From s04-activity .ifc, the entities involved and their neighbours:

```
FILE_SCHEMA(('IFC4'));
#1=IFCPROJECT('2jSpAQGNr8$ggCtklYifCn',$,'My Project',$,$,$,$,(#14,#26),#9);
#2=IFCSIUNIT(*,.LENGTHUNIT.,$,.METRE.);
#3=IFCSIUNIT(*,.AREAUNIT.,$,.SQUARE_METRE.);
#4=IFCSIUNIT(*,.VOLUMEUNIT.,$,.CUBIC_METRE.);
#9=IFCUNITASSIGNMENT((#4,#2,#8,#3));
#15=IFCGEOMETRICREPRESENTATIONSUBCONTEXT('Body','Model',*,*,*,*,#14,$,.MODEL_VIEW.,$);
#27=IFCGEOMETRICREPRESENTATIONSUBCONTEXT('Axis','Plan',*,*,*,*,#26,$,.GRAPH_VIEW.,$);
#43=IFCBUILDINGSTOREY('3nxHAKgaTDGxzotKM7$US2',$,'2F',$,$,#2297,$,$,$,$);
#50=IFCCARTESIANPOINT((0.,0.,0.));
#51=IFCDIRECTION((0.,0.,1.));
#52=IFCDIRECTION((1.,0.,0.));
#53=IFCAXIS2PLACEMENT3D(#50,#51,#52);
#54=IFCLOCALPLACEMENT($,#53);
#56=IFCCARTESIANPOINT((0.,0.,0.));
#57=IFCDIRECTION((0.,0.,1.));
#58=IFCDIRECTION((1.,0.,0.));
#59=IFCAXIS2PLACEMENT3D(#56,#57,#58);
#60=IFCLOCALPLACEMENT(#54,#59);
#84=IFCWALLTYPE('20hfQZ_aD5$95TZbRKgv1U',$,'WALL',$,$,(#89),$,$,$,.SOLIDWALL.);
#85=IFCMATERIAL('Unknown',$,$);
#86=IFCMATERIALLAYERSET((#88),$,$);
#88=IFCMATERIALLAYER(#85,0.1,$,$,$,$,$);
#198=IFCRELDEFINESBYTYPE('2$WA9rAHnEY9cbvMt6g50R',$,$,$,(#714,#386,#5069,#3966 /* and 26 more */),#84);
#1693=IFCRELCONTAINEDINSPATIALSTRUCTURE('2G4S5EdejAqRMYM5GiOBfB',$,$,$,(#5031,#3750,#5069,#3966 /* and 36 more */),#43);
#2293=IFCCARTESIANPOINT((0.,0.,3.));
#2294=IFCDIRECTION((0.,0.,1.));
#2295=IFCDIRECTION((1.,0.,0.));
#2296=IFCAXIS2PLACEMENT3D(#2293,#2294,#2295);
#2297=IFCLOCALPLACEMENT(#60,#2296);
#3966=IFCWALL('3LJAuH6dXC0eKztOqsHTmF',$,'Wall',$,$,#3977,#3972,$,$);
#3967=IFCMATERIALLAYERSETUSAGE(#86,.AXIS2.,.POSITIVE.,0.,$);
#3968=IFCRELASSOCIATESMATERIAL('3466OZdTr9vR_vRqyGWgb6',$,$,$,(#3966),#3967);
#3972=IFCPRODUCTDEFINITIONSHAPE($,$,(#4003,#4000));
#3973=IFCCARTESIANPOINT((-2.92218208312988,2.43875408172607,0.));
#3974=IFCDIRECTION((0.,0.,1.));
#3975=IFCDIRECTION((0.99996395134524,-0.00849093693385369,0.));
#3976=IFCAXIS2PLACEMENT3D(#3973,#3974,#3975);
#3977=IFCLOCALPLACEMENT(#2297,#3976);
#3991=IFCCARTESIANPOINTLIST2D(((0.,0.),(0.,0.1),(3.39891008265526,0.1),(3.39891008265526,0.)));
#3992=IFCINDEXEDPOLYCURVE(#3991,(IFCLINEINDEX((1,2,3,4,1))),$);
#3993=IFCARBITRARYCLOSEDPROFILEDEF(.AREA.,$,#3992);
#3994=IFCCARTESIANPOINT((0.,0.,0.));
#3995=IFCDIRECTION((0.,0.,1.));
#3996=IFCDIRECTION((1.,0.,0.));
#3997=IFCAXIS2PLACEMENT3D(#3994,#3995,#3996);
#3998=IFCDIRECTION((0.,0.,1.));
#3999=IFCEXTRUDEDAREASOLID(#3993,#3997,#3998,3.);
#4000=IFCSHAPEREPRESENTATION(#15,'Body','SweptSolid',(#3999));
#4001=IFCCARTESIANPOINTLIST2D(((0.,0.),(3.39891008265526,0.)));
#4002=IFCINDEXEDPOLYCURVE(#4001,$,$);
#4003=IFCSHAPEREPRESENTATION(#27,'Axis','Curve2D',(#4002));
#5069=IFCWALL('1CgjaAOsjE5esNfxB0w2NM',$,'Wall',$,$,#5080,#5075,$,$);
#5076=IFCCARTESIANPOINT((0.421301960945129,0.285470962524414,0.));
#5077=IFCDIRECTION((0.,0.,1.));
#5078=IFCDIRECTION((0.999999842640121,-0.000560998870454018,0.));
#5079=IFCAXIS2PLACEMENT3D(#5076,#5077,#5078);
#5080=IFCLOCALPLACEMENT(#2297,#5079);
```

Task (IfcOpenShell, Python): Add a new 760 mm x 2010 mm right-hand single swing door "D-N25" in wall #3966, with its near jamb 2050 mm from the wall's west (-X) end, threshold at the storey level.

```python
import numpy as np
import ifcopenshell
import ifcopenshell.api.feature
import ifcopenshell.api.geometry
import ifcopenshell.api.root
import ifcopenshell.api.spatial
import ifcopenshell.geom
import ifcopenshell.util.element
import ifcopenshell.util.placement
import ifcopenshell.util.representation
import ifcopenshell.util.shape
import ifcopenshell.util.unit

model = ifcopenshell.open("s04-activity .ifc")
unit_scale = ifcopenshell.util.unit.calculate_unit_scale(model)
settings = ifcopenshell.geom.settings()


def volume(element):
    """Net volume in cubic metres, openings subtracted."""
    shape = ifcopenshell.geom.create_shape(settings, element)
    return ifcopenshell.util.shape.get_volume(shape.geometry)


wall = model.by_guid("3LJAuH6dXC0eKztOqsHTmF")
storey = ifcopenshell.util.element.get_container(wall, ifc_class="IfcBuildingStorey")
context = ifcopenshell.util.representation.get_context(model, "Model", "Body", "MODEL_VIEW")
before = volume(wall)

width, height, from_end, sill = 0.76, 2.01, 2.05, 0.0  # metres

# The wall runs along its own X axis, and the end named is its -X end.
wall_shape = ifcopenshell.geom.create_shape(settings, wall)
x, y, z = ifcopenshell.util.shape.get_vertices(wall_shape.geometry).T
start = x.min() + from_end
face, thickness = float(y.min()), float(y.max() - y.min())
wall_matrix = ifcopenshell.util.placement.get_local_placement(wall.ObjectPlacement)
level = ifcopenshell.util.placement.get_local_placement(storey.ObjectPlacement)[2, 3]


def in_wall(x, y):
    """Placement at x, y metres in the wall's axes, at sill height."""
    matrix = wall_matrix.copy()
    matrix[:, 3] = wall_matrix @ np.array([x / unit_scale, y / unit_scale, 0.0, 1.0])
    matrix[2, 3] = level + sill / unit_scale
    return matrix


# Opening: a box that overshoots both wall faces by 50 mm.
opening = ifcopenshell.api.root.create_entity(model, ifc_class="IfcOpeningElement", predefined_type="OPENING")
box = ifcopenshell.api.geometry.add_wall_representation(
    model, context=context, length=width, height=height, thickness=thickness + 0.1
)
ifcopenshell.api.geometry.assign_representation(model, product=opening, representation=box)
ifcopenshell.api.geometry.edit_object_placement(model, product=opening, matrix=in_wall(start, face - 0.05), is_si=False)
ifcopenshell.api.feature.add_feature(model, feature=opening, element=wall)

door = ifcopenshell.api.root.create_entity(model, ifc_class="IfcDoor", name="D-N25", predefined_type="DOOR")
door.OverallWidth, door.OverallHeight = width / unit_scale, height / unit_scale
door.OperationType = "SINGLE_SWING_RIGHT"
body = ifcopenshell.api.geometry.add_door_representation(
    model,
    context=context,
    overall_width=door.OverallWidth,
    overall_height=door.OverallHeight,
    operation_type="SINGLE_SWING_RIGHT",
    lining_properties={"LiningDepth": thickness / unit_scale, "ThresholdDepth": thickness / unit_scale},
)
ifcopenshell.api.geometry.assign_representation(model, product=door, representation=body)
ifcopenshell.api.spatial.assign_container(model, products=[door], relating_structure=storey)
ifcopenshell.api.feature.add_filling(model, opening=opening, element=door)

# The lining spans the wall, so the door starts at the wall face.
ifcopenshell.api.geometry.edit_object_placement(model, product=door, matrix=in_wall(start, face), is_si=False)

after = volume(wall)

print(f"wall volume {before:.3f} -> {after:.3f} m3")

model.write("s04-activity _rev.ifc")
```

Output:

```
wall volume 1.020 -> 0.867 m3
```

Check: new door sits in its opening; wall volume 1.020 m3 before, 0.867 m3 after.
